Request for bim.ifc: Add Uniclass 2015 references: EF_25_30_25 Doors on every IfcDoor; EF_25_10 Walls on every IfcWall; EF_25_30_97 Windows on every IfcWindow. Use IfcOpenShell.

First a look at what the model holds.

```python
import ifcopenshell

model = ifcopenshell.open("bim.ifc")
print(model.schema)
print("classifications:", [c.Name for c in model.by_type("IfcClassification")])
for ifc_class in ("IfcDoor", "IfcRoof", "IfcStair", "IfcWall", "IfcWindow"):
    print(ifc_class, len(model.by_type(ifc_class)))
```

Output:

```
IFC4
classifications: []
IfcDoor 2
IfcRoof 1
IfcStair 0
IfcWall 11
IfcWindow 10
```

```python
import ifcopenshell
import ifcopenshell.api.classification

model = ifcopenshell.open("bim.ifc")

system = ifcopenshell.api.classification.add_classification(model, classification="Uniclass 2015")

codes = {
    "IfcDoor": ("EF_25_30_25", "Doors"),
    "IfcWall": ("EF_25_10", "Walls"),
    "IfcWindow": ("EF_25_30_97", "Windows"),
}
for ifc_class, (code, name) in codes.items():
    products = model.by_type(ifc_class)
    ifcopenshell.api.classification.add_reference(
        model, products=products, classification=system, identification=code, name=name
    )
    print(code, len(products))

model.write("bim_rev.ifc")
```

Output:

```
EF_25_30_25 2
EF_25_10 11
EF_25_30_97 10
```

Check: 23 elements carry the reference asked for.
